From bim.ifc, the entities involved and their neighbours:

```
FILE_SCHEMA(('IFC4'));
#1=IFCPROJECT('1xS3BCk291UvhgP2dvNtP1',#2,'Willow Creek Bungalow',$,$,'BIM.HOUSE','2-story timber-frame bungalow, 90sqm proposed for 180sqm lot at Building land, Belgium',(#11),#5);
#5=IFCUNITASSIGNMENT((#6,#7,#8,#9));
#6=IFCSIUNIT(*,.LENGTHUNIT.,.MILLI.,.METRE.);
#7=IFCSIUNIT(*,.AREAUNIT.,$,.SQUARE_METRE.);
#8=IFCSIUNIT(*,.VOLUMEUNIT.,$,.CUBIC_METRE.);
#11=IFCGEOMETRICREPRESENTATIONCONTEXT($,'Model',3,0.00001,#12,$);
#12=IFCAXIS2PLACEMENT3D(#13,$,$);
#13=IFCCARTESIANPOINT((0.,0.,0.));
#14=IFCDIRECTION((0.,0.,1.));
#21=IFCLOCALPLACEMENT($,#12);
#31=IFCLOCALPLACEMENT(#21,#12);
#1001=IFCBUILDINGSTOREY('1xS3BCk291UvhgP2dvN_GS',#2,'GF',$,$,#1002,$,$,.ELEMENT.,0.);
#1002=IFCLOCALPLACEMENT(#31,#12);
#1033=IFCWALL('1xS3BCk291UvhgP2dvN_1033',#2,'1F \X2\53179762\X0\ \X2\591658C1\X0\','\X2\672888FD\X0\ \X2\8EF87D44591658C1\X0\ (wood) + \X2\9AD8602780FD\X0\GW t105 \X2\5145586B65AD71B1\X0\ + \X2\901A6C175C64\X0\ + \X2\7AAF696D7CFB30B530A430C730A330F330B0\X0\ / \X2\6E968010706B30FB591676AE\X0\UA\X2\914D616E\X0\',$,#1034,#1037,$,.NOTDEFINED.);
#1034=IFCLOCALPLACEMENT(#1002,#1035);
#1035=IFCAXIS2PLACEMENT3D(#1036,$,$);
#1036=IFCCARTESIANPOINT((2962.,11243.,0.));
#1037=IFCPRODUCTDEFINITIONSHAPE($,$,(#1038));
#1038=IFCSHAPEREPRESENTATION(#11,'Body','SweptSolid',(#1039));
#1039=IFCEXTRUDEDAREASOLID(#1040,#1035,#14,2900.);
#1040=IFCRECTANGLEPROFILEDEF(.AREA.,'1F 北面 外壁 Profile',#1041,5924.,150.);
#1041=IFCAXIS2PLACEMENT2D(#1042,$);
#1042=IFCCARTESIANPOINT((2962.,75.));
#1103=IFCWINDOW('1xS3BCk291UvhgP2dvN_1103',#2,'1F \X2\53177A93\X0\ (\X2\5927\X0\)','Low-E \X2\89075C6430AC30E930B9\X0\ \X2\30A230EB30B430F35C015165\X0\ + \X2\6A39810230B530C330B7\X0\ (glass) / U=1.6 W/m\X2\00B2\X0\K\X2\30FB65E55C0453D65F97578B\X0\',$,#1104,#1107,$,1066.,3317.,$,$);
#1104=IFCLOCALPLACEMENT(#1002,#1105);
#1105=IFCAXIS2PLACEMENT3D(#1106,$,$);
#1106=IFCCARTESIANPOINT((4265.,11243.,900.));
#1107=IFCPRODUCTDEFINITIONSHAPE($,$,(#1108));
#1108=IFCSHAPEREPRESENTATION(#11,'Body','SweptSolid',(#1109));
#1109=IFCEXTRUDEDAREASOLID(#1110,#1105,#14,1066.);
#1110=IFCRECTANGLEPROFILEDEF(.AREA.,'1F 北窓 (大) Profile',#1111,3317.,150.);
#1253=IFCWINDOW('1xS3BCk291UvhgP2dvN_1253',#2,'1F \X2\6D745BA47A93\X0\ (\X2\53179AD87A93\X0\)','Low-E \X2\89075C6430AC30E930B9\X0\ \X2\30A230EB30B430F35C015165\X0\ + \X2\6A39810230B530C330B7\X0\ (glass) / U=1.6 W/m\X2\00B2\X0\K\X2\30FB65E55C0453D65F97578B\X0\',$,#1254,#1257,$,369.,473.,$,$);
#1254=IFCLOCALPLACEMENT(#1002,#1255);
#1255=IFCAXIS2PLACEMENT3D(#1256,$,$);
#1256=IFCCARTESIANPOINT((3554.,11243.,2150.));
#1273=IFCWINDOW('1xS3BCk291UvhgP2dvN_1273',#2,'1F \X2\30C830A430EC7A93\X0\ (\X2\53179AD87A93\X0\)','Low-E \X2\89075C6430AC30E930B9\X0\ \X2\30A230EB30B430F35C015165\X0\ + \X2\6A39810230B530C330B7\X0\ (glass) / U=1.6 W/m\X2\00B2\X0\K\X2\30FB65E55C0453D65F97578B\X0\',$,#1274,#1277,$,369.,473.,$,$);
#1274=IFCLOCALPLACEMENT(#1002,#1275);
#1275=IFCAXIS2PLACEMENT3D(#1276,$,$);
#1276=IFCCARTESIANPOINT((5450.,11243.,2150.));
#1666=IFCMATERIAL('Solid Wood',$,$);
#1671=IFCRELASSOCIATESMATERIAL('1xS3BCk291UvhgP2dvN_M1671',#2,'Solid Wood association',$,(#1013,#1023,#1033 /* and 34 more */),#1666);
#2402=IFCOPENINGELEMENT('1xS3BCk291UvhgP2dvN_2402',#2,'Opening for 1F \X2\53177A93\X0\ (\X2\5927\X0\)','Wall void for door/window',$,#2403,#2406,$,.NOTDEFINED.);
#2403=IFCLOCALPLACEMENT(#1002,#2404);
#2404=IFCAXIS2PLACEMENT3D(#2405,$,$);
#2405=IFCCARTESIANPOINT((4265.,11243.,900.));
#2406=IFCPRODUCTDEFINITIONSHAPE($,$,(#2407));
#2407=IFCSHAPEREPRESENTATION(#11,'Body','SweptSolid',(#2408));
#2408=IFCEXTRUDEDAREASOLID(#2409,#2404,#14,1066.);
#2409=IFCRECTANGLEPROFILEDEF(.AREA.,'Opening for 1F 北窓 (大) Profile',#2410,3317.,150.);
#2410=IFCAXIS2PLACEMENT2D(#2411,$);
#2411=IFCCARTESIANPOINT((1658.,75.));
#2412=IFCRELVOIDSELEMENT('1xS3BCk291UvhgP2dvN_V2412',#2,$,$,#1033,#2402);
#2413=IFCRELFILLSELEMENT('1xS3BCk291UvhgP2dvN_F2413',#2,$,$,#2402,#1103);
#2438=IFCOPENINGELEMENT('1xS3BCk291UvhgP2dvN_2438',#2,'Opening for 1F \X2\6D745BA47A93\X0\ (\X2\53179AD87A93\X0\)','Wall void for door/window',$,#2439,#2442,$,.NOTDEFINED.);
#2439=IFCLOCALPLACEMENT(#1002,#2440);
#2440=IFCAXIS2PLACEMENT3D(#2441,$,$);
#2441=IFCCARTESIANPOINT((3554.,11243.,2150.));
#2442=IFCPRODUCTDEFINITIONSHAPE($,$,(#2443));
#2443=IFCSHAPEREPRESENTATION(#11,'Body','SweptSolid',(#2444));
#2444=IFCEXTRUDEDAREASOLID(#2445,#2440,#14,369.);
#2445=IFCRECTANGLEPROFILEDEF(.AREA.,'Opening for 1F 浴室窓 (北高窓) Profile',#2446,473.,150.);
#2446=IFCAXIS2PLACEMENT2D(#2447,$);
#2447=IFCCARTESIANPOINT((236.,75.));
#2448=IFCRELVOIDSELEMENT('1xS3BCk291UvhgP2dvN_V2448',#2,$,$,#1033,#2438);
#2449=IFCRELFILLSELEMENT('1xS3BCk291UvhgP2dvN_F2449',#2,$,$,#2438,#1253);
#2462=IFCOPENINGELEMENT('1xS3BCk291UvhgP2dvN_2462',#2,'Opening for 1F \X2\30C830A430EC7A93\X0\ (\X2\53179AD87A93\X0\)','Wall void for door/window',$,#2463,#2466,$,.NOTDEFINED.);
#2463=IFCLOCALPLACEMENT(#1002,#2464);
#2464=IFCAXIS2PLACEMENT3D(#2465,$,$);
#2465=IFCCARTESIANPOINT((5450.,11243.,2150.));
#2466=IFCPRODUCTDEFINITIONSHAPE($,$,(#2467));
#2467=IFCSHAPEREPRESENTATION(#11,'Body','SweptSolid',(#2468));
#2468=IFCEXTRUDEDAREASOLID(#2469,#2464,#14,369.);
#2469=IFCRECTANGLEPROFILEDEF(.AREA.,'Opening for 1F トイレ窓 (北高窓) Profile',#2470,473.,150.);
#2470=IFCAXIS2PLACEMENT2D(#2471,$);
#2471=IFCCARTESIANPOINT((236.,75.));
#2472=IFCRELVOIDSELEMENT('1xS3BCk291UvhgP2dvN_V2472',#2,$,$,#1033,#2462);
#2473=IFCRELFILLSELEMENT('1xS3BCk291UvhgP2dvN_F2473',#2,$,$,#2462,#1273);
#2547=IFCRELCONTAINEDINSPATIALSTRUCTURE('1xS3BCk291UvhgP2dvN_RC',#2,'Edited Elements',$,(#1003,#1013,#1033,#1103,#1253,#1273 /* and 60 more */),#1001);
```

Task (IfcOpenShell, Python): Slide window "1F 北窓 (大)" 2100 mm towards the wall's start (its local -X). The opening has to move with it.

```python
import ifcopenshell
import ifcopenshell.api.geometry
import ifcopenshell.util.placement

model = ifcopenshell.open("bim.ifc")

window = model.by_id(1103)
opening = window.FillsVoids[0].RelatingOpeningElement
wall = opening.VoidsElements[0].RelatingBuildingElement

wall_matrix = ifcopenshell.util.placement.get_local_placement(wall.ObjectPlacement)
shift = wall_matrix[:3, 0] * -2100.0
before = ifcopenshell.util.placement.get_local_placement(window.ObjectPlacement)[:3, 3].copy()

# The window is not placed relative to its opening, so move both.
for product in (opening, window):
    matrix = ifcopenshell.util.placement.get_local_placement(product.ObjectPlacement)
    matrix[:3, 3] += shift
    ifcopenshell.api.geometry.edit_object_placement(model, product=product, matrix=matrix, is_si=False)

after = ifcopenshell.util.placement.get_local_placement(window.ObjectPlacement)[:3, 3]
print("window moved by", (after - before).round(3) + 0.0)

model.write("bim_edited.ifc")
```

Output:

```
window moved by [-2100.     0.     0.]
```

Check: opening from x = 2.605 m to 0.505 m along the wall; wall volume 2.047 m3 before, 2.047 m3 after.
